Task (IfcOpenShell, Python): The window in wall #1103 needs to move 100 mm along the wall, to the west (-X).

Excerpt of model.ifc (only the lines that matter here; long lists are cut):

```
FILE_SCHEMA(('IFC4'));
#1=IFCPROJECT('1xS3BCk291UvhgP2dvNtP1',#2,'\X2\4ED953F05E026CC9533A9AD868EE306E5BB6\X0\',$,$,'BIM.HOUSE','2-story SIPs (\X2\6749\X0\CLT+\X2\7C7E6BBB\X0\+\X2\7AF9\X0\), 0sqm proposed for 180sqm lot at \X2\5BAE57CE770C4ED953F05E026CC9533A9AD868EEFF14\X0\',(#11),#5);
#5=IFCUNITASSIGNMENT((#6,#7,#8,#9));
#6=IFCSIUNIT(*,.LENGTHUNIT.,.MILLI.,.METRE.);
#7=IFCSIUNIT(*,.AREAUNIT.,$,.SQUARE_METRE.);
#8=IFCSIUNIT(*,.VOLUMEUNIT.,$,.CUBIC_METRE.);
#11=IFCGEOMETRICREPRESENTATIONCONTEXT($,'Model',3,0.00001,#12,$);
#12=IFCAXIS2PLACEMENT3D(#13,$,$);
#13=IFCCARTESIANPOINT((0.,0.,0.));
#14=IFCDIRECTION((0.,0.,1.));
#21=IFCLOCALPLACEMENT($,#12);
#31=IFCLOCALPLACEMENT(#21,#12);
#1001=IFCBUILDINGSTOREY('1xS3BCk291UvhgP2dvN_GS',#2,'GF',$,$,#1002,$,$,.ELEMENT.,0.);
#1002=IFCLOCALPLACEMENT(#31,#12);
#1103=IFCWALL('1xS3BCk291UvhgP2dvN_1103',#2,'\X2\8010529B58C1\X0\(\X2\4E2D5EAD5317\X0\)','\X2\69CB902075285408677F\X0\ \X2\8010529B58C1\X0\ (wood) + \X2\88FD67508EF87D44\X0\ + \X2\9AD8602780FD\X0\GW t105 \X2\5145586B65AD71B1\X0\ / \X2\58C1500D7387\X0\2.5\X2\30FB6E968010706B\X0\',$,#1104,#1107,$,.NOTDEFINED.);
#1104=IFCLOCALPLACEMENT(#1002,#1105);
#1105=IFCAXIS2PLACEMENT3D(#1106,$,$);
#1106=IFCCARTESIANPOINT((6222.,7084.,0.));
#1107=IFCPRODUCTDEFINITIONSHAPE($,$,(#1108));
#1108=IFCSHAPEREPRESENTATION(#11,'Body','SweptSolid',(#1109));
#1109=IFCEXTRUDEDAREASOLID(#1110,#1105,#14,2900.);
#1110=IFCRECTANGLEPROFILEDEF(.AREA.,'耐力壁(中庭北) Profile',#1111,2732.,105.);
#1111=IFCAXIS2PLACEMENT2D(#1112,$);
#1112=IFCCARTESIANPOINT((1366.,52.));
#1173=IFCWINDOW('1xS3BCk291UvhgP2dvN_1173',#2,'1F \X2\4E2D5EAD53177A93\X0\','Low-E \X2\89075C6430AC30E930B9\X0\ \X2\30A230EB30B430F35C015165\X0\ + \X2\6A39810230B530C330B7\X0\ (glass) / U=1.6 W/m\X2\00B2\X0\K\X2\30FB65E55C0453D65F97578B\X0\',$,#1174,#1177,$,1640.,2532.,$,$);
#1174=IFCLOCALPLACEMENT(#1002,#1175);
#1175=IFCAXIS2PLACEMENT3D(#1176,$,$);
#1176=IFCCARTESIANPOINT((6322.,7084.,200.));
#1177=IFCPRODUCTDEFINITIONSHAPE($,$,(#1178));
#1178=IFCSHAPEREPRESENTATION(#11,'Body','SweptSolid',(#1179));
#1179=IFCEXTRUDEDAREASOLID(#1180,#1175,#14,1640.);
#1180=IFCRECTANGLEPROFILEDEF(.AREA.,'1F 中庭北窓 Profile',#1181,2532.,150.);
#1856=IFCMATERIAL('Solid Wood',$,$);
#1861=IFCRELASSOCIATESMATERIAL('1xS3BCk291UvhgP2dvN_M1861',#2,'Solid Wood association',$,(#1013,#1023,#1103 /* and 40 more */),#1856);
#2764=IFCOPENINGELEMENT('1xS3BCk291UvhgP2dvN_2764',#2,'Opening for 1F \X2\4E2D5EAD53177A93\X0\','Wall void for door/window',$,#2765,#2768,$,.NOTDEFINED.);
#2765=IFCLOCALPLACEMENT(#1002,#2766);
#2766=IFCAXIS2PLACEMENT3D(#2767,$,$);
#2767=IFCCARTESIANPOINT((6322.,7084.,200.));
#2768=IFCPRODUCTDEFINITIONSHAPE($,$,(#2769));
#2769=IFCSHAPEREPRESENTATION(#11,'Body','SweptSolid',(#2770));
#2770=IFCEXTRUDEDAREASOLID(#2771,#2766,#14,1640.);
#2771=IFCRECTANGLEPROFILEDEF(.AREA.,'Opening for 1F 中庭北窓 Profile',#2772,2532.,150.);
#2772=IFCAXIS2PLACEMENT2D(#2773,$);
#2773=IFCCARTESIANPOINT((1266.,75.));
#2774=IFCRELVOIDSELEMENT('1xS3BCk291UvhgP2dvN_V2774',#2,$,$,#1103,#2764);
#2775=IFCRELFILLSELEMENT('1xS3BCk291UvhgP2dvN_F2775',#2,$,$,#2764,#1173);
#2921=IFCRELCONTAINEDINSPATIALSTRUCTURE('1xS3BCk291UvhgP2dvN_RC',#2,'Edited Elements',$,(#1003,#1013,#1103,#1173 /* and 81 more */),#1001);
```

```python
import ifcopenshell
import ifcopenshell.api.geometry
import ifcopenshell.util.placement

model = ifcopenshell.open("model.ifc")

window = model.by_guid("1xS3BCk291UvhgP2dvN_1173")
opening = window.FillsVoids[0].RelatingOpeningElement
wall = opening.VoidsElements[0].RelatingBuildingElement

wall_matrix = ifcopenshell.util.placement.get_local_placement(wall.ObjectPlacement)
shift = wall_matrix[:3, 0] * -100.0
before = ifcopenshell.util.placement.get_local_placement(window.ObjectPlacement)[:3, 3].copy()

# The window is not placed relative to its opening, so move both.
for product in (opening, window):
    matrix = ifcopenshell.util.placement.get_local_placement(product.ObjectPlacement)
    matrix[:3, 3] += shift
    ifcopenshell.api.geometry.edit_object_placement(model, product=product, matrix=matrix, is_si=False)

after = ifcopenshell.util.placement.get_local_placement(window.ObjectPlacement)[:3, 3]
print("window moved by", (after - before).round(3) + 0.0)

model.write("model_updated.ifc")
```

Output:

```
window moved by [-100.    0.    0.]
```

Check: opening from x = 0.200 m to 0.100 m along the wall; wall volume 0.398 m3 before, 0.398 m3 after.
